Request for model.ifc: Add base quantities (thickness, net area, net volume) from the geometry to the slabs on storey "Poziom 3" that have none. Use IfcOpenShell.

First a look at what the model holds.

```python
import ifcopenshell
import ifcopenshell.util.element
import ifcopenshell.util.unit

model = ifcopenshell.open("model.ifc")
print(model.schema)
for unit_type in ("LENGTHUNIT", "AREAUNIT", "VOLUMEUNIT"):
    print(unit_type, ifcopenshell.util.unit.calculate_unit_scale(model, unit_type))
storey = next(s for s in model.by_type("IfcBuildingStorey") if s.Name == "Poziom 3")
slabs = [e for e in ifcopenshell.util.element.get_decomposition(storey) if e.is_a("IfcSlab")]
for e in sorted(slabs, key=lambda e: e.id()):
    print(e.id(), e.is_a(), e.Name, list(ifcopenshell.util.element.get_psets(e, qtos_only=True)), sep=" | ")
```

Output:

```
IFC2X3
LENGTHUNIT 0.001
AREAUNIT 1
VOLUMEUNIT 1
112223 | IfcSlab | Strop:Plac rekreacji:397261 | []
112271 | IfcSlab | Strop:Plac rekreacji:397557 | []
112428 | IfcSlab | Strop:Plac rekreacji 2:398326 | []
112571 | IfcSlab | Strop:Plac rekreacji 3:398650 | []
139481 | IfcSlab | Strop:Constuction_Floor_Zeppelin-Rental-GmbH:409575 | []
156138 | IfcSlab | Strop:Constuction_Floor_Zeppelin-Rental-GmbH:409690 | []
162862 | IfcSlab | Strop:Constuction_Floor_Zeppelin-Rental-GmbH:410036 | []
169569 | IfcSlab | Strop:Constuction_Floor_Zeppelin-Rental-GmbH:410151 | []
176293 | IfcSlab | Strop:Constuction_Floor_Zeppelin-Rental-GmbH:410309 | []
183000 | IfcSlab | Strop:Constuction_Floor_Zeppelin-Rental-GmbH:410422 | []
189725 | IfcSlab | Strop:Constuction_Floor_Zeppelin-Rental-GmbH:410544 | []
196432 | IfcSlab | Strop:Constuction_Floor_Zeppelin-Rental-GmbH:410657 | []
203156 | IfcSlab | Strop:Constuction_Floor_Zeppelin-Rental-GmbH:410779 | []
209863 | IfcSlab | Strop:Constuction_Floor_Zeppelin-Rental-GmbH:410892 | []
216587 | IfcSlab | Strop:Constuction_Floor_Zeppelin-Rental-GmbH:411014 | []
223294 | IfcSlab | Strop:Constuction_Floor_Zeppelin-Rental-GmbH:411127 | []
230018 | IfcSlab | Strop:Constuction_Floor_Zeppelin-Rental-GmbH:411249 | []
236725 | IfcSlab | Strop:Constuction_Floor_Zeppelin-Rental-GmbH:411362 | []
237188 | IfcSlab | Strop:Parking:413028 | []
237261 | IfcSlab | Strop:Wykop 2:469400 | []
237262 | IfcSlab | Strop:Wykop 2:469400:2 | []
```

```python
import ifcopenshell
import ifcopenshell.api.pset
import ifcopenshell.geom
import ifcopenshell.util.element
import ifcopenshell.util.shape
import ifcopenshell.util.unit

model = ifcopenshell.open("model.ifc")
unit_scale = ifcopenshell.util.unit.calculate_unit_scale(model)
area_scale = ifcopenshell.util.unit.calculate_unit_scale(model, "AREAUNIT")
volume_scale = ifcopenshell.util.unit.calculate_unit_scale(model, "VOLUMEUNIT")
settings = ifcopenshell.geom.settings()

storey = next(s for s in model.by_type("IfcBuildingStorey") if s.Name == "Poziom 3")
slabs = [e for e in ifcopenshell.util.element.get_decomposition(storey) if e.is_a("IfcSlab")]

for e in sorted(slabs, key=lambda e: e.id()):
    if ifcopenshell.util.element.get_psets(e, qtos_only=True, should_inherit=False):
        continue
    # Geometry comes back in metres, in the element's own axes.
    shape = ifcopenshell.geom.create_shape(settings, e)
    values = {
        "Width": ifcopenshell.util.shape.get_z(shape.geometry) / unit_scale,
        "NetArea": ifcopenshell.util.shape.get_footprint_area(shape.geometry) / area_scale,
        "NetVolume": ifcopenshell.util.shape.get_volume(shape.geometry) / volume_scale,
    }
    qto = ifcopenshell.api.pset.add_qto(model, product=e, name="BaseQuantities")
    ifcopenshell.api.pset.edit_qto(model, qto=qto, properties=values)
    print(e.id(), {k: round(v, 3) for k, v in values.items()})

model.write("model_updated.ifc")
```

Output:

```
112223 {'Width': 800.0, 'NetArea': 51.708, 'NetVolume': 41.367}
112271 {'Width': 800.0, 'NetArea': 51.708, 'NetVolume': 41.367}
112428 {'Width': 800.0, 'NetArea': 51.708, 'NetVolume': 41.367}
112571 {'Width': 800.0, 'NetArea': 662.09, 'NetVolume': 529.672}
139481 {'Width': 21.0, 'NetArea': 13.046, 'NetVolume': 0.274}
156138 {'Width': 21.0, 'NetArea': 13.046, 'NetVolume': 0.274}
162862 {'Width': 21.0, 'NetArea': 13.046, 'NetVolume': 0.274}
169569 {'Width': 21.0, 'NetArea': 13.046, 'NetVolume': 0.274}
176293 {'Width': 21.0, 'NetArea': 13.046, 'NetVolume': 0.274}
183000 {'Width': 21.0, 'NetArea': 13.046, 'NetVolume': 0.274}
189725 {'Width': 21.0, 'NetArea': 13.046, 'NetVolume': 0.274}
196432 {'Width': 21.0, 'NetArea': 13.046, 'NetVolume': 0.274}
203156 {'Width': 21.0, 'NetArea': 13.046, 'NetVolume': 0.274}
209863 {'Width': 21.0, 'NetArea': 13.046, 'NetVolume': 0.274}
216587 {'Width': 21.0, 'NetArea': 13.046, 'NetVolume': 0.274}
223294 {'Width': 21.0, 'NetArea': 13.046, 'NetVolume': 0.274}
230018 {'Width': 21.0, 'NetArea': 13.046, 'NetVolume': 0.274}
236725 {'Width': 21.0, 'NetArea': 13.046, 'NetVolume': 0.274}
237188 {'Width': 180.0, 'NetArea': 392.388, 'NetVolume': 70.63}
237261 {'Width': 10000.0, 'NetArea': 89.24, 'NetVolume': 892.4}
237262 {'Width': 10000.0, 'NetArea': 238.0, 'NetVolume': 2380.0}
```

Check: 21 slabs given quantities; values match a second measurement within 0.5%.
